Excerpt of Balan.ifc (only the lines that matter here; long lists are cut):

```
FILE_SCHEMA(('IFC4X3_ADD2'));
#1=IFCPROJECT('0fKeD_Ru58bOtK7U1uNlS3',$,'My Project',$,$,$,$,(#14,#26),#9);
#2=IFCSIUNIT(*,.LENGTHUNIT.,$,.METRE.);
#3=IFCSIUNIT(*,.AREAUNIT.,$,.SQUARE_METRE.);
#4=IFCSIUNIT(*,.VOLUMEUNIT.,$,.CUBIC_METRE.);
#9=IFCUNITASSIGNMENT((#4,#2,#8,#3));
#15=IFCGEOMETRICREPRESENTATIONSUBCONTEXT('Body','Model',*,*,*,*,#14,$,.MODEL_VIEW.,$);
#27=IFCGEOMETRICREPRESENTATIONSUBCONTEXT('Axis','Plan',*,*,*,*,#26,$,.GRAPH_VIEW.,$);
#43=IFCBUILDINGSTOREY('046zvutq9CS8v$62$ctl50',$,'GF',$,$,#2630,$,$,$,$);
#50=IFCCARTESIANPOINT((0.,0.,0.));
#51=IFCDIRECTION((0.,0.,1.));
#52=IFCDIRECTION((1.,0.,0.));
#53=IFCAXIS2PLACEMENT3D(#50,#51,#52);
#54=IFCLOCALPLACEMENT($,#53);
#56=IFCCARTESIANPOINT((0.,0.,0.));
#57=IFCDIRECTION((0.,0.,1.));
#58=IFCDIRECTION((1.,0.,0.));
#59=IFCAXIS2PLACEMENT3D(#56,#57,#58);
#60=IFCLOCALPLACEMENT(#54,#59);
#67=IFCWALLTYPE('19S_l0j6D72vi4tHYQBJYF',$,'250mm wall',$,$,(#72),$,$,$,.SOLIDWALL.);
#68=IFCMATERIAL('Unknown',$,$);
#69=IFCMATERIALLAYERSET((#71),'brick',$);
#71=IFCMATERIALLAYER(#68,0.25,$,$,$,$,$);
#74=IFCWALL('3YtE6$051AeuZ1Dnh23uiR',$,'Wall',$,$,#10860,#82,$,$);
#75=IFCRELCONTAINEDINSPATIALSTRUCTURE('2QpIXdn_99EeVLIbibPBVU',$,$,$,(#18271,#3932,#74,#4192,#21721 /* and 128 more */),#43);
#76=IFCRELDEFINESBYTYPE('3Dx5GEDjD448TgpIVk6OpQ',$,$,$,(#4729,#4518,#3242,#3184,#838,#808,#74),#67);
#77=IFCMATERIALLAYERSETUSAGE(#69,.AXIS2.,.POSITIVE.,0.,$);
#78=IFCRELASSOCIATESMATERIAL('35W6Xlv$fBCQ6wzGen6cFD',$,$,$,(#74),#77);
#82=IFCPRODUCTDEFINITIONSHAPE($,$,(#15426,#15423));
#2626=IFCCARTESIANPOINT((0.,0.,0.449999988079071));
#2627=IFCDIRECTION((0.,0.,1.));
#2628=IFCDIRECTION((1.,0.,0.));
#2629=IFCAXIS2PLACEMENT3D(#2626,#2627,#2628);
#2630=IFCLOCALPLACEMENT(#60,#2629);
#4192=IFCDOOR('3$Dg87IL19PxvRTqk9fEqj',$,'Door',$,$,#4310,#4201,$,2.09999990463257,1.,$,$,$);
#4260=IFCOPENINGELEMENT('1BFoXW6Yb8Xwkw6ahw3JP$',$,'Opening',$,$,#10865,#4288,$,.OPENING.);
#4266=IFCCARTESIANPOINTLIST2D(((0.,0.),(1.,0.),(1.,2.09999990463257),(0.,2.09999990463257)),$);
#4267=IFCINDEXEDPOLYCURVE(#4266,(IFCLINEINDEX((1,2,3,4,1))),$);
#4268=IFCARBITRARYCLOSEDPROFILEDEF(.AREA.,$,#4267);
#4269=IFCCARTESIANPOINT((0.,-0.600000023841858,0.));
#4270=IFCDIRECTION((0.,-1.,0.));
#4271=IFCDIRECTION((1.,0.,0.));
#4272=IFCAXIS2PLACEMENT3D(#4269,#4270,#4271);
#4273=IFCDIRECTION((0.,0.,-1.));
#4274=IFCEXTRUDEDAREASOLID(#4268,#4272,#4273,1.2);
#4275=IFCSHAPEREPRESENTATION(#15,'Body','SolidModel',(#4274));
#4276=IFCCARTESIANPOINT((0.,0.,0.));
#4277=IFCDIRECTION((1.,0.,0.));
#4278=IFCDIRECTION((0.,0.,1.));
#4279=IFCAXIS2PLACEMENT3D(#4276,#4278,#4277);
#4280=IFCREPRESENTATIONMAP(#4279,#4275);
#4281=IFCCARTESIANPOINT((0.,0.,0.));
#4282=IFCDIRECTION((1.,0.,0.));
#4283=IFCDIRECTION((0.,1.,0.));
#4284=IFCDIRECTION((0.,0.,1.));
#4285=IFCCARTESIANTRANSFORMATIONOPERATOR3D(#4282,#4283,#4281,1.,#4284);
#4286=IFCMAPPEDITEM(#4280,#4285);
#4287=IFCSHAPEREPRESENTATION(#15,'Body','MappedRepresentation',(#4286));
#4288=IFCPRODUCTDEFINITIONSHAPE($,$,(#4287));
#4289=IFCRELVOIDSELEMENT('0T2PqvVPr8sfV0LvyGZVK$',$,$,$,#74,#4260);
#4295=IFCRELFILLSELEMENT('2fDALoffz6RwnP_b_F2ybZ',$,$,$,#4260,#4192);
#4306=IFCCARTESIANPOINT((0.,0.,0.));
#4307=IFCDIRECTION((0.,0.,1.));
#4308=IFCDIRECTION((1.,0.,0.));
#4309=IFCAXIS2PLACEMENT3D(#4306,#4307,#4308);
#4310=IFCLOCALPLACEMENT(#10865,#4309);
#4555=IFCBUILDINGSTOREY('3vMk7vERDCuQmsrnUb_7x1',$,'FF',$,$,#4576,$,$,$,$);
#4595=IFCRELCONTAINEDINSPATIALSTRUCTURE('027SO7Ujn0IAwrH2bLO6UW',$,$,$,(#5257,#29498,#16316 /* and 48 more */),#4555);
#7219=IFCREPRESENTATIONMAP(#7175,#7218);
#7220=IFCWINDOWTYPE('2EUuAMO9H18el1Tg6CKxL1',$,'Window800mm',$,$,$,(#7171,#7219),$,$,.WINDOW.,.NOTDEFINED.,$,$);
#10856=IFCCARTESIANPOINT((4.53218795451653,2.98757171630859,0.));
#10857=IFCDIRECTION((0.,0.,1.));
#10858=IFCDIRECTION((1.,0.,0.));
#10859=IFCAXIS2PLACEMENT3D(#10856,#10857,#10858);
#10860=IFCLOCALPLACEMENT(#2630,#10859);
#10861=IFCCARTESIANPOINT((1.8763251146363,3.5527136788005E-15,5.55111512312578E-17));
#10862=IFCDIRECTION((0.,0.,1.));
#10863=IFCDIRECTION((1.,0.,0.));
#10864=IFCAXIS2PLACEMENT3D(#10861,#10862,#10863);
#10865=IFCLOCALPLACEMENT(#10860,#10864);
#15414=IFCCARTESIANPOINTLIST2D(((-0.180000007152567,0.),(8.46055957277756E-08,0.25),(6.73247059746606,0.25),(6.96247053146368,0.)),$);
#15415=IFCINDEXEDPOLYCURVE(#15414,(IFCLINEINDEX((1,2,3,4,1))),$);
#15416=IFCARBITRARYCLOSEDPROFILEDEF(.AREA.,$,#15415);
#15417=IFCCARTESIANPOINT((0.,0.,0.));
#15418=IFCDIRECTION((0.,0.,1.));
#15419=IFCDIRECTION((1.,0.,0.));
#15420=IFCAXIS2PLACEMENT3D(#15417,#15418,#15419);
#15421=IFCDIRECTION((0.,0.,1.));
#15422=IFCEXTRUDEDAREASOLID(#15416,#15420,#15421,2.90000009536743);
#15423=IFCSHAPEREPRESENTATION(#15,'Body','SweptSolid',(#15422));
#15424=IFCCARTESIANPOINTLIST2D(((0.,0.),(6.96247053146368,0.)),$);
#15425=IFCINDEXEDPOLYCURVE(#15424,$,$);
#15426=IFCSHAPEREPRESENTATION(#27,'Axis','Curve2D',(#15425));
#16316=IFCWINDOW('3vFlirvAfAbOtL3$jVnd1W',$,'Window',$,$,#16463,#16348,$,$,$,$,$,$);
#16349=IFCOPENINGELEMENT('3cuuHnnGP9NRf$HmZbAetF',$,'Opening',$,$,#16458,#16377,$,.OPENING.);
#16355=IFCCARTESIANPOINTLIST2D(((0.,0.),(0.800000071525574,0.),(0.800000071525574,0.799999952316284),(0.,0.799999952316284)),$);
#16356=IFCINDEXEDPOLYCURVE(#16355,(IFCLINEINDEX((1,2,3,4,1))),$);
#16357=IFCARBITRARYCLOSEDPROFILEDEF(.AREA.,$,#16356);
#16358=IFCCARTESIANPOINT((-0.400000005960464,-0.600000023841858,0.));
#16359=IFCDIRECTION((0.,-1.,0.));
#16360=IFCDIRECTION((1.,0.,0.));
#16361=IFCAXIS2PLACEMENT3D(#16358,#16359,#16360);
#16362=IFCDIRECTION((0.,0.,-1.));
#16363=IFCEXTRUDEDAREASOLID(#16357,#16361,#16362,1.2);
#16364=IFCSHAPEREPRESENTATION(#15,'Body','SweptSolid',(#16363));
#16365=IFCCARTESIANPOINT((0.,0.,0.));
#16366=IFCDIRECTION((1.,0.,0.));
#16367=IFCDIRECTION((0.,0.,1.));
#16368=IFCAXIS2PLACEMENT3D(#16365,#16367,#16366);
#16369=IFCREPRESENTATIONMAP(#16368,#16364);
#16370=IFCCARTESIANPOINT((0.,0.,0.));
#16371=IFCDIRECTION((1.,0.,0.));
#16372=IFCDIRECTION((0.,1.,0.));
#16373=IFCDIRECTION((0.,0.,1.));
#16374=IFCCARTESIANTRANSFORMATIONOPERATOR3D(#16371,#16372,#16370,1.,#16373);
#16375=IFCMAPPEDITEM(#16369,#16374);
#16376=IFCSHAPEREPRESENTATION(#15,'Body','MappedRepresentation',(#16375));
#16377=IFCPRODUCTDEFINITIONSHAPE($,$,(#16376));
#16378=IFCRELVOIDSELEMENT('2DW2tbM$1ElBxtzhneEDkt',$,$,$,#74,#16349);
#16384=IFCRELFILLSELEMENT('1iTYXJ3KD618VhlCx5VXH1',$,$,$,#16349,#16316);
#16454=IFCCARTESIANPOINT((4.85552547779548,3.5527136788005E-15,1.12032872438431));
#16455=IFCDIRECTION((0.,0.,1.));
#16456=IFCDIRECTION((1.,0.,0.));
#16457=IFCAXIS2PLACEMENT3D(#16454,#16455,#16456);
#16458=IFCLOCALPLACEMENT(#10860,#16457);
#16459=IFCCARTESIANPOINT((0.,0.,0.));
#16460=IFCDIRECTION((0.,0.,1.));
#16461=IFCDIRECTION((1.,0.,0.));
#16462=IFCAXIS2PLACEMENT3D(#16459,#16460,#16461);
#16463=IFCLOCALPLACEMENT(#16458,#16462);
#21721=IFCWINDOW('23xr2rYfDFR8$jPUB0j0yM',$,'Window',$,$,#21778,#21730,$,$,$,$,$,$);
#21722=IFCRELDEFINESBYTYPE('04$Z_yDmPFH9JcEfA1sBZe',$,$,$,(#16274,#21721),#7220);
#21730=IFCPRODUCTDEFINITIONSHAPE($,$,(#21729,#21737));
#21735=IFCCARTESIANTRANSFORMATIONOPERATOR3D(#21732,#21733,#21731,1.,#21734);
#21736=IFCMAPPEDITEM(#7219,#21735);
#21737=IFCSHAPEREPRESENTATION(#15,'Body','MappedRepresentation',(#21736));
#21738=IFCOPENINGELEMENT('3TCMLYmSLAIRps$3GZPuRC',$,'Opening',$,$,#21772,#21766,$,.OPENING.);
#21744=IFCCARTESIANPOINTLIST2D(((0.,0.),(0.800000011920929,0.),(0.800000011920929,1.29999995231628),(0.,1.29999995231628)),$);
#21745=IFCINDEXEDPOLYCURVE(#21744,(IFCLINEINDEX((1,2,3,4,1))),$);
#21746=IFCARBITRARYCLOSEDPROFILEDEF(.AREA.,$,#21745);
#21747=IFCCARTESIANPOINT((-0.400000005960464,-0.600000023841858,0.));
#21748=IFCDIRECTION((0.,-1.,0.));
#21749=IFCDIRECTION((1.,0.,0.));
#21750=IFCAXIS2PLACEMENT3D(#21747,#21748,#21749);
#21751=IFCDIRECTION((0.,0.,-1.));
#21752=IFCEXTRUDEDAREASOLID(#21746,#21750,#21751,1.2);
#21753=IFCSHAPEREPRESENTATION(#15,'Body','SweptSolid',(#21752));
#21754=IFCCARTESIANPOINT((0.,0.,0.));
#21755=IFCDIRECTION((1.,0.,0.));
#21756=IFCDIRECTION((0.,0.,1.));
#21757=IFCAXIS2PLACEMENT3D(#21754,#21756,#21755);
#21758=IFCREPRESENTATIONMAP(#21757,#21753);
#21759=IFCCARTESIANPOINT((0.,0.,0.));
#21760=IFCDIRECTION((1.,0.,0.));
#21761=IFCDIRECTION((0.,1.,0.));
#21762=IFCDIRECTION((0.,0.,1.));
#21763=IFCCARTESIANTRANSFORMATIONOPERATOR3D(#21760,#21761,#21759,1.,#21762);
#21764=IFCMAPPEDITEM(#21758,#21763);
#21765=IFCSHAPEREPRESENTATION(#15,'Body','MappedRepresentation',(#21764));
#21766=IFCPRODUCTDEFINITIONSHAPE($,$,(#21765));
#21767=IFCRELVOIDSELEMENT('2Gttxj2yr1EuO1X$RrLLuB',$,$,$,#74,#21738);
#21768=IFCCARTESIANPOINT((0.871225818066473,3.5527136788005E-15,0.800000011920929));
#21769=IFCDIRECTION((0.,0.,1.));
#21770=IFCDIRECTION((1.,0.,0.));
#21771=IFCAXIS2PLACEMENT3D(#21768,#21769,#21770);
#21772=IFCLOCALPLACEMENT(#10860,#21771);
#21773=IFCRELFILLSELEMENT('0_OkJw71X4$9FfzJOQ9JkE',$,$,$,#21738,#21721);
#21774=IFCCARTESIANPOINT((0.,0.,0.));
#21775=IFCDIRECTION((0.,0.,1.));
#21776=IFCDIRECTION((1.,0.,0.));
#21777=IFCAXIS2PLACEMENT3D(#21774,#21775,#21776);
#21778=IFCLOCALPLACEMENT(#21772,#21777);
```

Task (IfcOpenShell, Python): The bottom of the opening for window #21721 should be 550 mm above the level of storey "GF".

```python
import numpy as np
import ifcopenshell
import ifcopenshell.api.geometry
import ifcopenshell.geom
import ifcopenshell.util.element
import ifcopenshell.util.placement
import ifcopenshell.util.shape
import ifcopenshell.util.unit

model = ifcopenshell.open("Balan.ifc")
unit_scale = ifcopenshell.util.unit.calculate_unit_scale(model)

window = model.by_guid("23xr2rYfDFR8$jPUB0j0yM")
opening = window.FillsVoids[0].RelatingOpeningElement
storey = ifcopenshell.util.element.get_container(window, ifc_class="IfcBuildingStorey")
level = ifcopenshell.util.placement.get_local_placement(storey.ObjectPlacement)[2, 3]

# The opening's origin need not be at the sill, so measure its lowest point.
shape = ifcopenshell.geom.create_shape(ifcopenshell.geom.settings(), opening)
bottom = ifcopenshell.util.shape.get_shape_bottom_elevation(shape, shape.geometry) / unit_scale
dz = level + 0.55 / unit_scale - bottom

shift = np.array([0.0, 0.0, dz])
# The window is placed relative to its opening, so it follows when the opening moves.
matrix = ifcopenshell.util.placement.get_local_placement(opening.ObjectPlacement)
matrix[:3, 3] += shift
ifcopenshell.api.geometry.edit_object_placement(
    model, product=opening, matrix=matrix, is_si=False, should_transform_children=True
)

print(f"moved by {dz * unit_scale:+.3f} m")

model.write("Balan-out.ifc")
```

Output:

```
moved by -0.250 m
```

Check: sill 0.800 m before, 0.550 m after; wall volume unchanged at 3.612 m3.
